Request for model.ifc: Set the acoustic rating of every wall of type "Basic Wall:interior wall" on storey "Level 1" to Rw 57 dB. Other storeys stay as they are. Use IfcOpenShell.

First a look at what the model holds.

```python
import ifcopenshell
import ifcopenshell.util.element

model = ifcopenshell.open("model.ifc")
print(model.schema)
storey = next(s for s in model.by_type("IfcBuildingStorey") if s.Name == "Level 1")
walls = [e for e in ifcopenshell.util.element.get_decomposition(storey) if e.is_a("IfcWall")]
seen = {}
for e in walls:
    element_type = ifcopenshell.util.element.get_type(e)
    key = (element_type.Name if element_type != e and element_type else None, ifcopenshell.util.element.get_pset(e, "Pset_WallCommon", "AcousticRating"))
    seen[key] = seen.get(key, 0) + 1
for (name, value), count in sorted(seen.items(), key=str):
    print(count, "x", name, "|", value)
```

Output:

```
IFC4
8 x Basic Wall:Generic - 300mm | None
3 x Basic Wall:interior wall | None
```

```python
import ifcopenshell
import ifcopenshell.api.pset
import ifcopenshell.util.element

model = ifcopenshell.open("model.ifc")

storey = next(s for s in model.by_type("IfcBuildingStorey") if s.Name == "Level 1")
walls = [e for e in ifcopenshell.util.element.get_decomposition(storey) if e.is_a("IfcWall")]

count = 0
for e in walls:
    element_type = ifcopenshell.util.element.get_type(e)
    if element_type in (None, e) or element_type.Name != "Basic Wall:interior wall":
        continue
    # add_pset returns the element's existing set when there is one.
    pset = ifcopenshell.api.pset.add_pset(model, product=e, name="Pset_WallCommon")
    ifcopenshell.api.pset.edit_pset(model, pset=pset, properties={"AcousticRating": "Rw 57 dB"})
    count += 1

print(count, "walls updated")

model.write("model_v2.ifc")
```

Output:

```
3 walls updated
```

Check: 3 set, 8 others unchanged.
